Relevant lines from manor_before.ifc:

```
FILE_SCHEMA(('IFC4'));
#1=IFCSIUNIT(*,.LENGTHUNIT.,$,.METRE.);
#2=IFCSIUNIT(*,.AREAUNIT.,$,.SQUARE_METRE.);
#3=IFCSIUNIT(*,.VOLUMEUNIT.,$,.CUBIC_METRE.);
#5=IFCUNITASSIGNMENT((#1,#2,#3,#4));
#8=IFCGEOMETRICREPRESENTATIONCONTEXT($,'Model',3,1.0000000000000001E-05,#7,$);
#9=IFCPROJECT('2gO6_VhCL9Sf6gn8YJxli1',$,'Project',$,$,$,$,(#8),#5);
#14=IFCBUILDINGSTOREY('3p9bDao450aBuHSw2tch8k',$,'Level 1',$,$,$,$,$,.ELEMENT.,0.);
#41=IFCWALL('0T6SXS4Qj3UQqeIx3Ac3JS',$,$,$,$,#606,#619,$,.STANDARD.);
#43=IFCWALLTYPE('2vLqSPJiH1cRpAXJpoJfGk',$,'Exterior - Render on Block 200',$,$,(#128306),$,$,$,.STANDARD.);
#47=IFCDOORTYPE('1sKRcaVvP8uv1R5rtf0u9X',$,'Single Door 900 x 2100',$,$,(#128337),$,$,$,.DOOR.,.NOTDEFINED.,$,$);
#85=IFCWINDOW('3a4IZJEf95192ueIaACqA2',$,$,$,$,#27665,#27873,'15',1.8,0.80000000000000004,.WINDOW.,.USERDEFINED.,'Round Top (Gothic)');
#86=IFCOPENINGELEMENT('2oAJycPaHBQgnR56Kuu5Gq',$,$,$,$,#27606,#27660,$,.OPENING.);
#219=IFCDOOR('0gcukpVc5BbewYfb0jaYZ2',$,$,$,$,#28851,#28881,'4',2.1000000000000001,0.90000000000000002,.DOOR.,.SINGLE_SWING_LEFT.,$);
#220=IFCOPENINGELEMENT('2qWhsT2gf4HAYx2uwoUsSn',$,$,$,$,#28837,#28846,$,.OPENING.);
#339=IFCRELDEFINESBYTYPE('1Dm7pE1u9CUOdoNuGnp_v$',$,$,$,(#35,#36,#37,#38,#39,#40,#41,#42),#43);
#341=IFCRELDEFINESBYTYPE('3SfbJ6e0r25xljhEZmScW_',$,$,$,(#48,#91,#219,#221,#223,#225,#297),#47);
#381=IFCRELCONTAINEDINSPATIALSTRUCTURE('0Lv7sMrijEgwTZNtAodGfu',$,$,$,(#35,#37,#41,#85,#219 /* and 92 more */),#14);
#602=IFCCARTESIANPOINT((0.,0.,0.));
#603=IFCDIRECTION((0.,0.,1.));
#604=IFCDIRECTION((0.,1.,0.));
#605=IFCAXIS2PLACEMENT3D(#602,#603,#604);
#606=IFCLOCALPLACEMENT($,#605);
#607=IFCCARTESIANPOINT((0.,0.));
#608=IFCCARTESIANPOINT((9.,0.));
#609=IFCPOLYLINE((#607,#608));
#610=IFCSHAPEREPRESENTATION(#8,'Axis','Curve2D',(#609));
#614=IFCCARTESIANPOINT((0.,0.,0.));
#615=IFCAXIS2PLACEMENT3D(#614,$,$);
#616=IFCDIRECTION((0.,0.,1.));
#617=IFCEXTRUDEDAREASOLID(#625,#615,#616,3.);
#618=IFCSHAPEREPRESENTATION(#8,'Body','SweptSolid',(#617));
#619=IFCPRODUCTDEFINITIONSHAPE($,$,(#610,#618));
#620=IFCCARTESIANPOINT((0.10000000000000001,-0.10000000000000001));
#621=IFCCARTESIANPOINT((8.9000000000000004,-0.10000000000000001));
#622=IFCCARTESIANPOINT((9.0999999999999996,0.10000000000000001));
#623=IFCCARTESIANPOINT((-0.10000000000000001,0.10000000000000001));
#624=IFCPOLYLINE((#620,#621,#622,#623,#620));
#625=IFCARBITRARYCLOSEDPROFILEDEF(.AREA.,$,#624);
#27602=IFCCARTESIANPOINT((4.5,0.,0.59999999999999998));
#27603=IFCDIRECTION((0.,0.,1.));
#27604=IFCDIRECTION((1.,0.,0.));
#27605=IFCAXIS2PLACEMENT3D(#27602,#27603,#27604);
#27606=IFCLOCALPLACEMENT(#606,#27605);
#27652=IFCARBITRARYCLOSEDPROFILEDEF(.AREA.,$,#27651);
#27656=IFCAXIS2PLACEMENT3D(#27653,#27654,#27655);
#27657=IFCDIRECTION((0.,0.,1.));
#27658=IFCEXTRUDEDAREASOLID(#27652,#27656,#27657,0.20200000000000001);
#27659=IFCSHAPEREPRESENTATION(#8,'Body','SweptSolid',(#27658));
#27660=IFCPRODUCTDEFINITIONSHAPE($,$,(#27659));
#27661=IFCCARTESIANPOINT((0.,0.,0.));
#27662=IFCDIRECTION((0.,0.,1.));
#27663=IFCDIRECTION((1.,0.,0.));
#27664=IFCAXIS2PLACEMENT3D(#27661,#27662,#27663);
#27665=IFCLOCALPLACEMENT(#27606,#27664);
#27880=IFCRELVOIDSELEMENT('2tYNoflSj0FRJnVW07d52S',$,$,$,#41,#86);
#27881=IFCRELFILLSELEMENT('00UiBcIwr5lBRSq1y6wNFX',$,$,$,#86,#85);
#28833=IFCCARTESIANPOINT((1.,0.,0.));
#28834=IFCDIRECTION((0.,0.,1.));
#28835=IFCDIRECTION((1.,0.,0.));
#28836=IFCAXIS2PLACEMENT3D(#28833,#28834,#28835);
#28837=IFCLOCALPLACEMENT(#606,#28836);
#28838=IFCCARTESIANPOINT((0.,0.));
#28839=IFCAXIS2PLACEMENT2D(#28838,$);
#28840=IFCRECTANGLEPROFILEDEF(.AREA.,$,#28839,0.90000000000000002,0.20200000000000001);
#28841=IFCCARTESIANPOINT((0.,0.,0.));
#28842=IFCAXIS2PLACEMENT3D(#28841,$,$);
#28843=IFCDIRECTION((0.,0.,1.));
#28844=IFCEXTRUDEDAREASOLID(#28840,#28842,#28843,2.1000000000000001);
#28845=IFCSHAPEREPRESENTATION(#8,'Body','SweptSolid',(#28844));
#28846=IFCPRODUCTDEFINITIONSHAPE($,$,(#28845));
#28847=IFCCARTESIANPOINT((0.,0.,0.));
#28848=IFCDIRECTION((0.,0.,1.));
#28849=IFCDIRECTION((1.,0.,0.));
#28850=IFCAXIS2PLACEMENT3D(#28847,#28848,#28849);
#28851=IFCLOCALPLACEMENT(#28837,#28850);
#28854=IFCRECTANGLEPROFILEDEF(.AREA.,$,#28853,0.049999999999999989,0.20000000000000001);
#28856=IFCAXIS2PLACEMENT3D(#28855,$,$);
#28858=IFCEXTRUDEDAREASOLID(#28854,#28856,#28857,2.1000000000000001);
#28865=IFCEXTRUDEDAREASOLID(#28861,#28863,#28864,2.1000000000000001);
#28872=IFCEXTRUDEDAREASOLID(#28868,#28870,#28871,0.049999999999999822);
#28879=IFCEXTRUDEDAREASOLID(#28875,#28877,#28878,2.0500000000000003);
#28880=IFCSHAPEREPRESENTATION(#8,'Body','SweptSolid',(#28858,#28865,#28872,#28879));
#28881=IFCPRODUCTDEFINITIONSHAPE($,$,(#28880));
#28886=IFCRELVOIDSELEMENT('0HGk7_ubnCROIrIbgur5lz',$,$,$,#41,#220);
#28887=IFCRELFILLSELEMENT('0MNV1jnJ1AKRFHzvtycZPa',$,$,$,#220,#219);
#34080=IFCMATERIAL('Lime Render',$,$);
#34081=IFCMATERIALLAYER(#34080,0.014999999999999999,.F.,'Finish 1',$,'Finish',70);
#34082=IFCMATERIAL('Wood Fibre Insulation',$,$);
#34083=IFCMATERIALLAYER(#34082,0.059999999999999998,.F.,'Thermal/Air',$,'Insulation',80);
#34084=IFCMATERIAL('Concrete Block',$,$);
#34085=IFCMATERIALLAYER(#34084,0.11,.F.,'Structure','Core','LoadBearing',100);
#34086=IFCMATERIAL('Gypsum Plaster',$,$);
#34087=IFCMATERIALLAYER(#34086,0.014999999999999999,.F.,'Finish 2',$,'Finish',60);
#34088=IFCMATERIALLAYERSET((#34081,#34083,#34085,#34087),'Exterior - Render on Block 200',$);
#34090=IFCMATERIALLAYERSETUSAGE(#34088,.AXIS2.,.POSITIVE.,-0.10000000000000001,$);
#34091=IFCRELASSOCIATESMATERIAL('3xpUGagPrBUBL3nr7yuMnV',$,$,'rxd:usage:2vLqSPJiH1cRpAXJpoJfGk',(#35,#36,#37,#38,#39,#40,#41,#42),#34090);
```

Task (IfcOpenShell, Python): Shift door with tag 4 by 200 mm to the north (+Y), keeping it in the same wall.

```python
import ifcopenshell
import ifcopenshell.api.geometry
import ifcopenshell.util.placement
import ifcopenshell.util.unit

model = ifcopenshell.open("manor_before.ifc")
unit_scale = ifcopenshell.util.unit.calculate_unit_scale(model)

door = model.by_guid("0gcukpVc5BbewYfb0jaYZ2")
opening = door.FillsVoids[0].RelatingOpeningElement
wall = opening.VoidsElements[0].RelatingBuildingElement

wall_matrix = ifcopenshell.util.placement.get_local_placement(wall.ObjectPlacement)
shift = wall_matrix[:3, 0] * 0.2 / unit_scale
before = ifcopenshell.util.placement.get_local_placement(door.ObjectPlacement)[:3, 3].copy()

# The door is placed relative to its opening, so it follows when the opening moves.
matrix = ifcopenshell.util.placement.get_local_placement(opening.ObjectPlacement)
matrix[:3, 3] += shift
ifcopenshell.api.geometry.edit_object_placement(
    model, product=opening, matrix=matrix, is_si=False, should_transform_children=True
)

after = ifcopenshell.util.placement.get_local_placement(door.ObjectPlacement)[:3, 3]
print("door moved by", (after - before).round(3) + 0.0)

model.write("manor_before-out.ifc")
```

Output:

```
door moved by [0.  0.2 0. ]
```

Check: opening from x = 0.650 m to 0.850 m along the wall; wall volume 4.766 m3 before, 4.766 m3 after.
